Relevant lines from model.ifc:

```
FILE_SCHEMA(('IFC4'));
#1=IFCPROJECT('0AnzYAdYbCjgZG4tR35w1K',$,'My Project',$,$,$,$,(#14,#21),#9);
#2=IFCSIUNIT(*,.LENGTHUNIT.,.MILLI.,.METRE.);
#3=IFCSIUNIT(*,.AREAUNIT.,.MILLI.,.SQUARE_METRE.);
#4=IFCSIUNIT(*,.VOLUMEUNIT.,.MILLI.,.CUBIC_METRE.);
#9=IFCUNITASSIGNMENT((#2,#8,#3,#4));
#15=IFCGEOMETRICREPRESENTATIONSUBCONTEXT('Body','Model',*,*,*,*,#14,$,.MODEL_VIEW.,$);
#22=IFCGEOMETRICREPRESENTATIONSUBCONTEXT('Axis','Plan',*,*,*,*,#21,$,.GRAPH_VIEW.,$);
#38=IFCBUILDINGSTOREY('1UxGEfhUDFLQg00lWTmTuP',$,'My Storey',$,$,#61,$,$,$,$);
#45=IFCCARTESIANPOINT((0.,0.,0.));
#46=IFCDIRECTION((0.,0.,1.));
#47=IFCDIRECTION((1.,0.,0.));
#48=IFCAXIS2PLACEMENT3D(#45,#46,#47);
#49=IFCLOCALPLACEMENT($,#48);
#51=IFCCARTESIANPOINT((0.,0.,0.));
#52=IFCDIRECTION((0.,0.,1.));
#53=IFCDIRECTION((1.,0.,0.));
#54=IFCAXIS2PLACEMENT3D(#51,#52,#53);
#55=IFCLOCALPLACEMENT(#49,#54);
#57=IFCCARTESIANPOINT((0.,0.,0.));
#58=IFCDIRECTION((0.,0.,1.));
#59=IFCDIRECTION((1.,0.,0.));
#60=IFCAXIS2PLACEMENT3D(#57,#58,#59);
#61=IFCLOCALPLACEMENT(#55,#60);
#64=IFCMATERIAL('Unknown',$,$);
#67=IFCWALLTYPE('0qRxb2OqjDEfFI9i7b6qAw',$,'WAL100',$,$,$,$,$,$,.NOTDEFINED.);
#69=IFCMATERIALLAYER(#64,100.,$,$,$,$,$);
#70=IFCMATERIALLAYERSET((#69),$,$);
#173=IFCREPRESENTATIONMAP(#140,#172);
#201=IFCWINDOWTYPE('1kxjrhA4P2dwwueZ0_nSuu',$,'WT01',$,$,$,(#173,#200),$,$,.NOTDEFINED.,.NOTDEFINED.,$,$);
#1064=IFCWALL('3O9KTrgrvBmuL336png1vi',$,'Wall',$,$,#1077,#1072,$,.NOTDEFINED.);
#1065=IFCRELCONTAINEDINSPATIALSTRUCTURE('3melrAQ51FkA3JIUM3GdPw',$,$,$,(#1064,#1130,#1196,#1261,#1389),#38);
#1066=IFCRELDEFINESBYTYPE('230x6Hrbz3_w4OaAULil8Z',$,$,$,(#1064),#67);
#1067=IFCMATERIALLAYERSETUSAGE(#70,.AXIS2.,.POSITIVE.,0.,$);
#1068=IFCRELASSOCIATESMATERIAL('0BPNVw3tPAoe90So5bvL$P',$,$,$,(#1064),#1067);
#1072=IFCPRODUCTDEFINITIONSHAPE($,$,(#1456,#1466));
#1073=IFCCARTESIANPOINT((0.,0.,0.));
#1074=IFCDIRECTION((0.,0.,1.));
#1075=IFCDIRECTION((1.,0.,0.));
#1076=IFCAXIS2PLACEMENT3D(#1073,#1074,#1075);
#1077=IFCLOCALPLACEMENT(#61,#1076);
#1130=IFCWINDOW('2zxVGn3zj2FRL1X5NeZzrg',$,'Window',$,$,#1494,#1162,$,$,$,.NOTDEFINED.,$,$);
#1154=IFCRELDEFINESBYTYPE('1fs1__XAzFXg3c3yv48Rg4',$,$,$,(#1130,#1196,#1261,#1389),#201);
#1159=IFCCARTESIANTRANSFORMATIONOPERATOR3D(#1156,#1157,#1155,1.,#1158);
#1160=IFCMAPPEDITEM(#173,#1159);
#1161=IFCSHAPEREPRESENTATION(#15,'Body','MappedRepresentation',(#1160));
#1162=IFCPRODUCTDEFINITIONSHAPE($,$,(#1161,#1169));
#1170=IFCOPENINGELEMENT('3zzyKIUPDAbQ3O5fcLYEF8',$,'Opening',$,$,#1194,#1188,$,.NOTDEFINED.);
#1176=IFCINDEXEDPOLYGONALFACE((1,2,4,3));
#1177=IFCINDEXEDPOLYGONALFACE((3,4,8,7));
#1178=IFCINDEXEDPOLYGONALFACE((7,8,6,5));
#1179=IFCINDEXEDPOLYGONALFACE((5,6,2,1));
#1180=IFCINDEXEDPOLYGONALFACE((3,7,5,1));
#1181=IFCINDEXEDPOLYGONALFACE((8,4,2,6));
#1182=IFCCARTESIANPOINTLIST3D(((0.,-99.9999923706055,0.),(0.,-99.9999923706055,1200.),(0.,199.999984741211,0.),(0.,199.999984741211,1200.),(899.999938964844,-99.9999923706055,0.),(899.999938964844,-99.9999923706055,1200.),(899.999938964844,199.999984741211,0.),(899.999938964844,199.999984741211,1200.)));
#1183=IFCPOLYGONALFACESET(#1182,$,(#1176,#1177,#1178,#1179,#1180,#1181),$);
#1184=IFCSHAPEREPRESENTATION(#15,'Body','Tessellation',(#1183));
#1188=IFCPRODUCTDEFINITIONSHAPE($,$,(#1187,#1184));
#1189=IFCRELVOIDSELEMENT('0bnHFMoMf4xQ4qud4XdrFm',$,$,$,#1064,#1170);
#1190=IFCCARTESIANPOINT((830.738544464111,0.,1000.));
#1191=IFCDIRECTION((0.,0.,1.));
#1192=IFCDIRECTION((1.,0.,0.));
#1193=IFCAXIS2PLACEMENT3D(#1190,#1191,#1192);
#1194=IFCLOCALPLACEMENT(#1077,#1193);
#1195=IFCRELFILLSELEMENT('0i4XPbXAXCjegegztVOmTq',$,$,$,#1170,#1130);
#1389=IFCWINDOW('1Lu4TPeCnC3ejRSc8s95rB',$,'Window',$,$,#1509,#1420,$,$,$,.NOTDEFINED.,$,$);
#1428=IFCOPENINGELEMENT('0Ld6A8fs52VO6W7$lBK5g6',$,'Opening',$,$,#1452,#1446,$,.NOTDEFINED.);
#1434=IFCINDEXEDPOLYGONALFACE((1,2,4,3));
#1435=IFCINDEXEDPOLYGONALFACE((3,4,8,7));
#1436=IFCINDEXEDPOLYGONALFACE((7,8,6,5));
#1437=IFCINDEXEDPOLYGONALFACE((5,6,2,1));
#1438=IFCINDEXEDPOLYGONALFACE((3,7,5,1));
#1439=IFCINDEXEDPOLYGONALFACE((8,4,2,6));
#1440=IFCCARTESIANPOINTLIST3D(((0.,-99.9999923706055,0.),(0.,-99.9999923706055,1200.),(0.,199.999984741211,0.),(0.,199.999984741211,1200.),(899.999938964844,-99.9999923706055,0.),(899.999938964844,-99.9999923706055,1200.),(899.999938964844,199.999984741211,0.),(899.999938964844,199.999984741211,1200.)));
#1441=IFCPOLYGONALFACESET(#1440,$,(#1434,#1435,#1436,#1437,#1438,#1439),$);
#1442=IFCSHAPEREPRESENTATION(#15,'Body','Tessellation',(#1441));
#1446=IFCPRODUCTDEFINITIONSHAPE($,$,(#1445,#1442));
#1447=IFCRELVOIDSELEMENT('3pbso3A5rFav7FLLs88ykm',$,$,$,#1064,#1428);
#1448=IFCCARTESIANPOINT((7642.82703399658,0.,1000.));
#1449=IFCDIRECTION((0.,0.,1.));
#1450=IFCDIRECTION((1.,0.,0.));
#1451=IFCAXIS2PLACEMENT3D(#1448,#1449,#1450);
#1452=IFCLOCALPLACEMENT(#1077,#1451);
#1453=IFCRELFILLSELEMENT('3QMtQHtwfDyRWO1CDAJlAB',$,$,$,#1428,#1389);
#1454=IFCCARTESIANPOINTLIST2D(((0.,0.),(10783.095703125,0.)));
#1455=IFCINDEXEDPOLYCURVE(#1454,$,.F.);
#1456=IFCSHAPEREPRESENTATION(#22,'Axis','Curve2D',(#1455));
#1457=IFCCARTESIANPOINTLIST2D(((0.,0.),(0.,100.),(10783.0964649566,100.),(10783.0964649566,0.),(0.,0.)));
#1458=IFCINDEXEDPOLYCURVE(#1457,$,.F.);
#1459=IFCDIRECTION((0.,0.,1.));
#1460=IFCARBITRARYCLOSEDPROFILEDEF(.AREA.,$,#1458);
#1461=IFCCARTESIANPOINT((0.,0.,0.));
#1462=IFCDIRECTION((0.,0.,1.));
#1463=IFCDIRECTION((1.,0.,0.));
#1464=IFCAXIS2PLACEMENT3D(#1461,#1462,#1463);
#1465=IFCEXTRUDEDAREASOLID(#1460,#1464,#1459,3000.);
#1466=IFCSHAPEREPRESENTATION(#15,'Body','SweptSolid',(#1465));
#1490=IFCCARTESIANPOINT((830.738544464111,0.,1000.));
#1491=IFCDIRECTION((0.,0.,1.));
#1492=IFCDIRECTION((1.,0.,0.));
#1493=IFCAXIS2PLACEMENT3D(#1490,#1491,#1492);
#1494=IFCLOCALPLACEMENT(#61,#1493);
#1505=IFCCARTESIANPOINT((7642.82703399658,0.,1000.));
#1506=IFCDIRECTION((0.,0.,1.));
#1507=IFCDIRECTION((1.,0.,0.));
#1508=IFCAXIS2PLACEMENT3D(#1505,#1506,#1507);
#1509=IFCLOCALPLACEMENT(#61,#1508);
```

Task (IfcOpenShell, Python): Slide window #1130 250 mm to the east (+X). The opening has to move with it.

```python
import ifcopenshell
import ifcopenshell.api.geometry
import ifcopenshell.util.placement

model = ifcopenshell.open("model.ifc")

window = model.by_guid("2zxVGn3zj2FRL1X5NeZzrg")
opening = window.FillsVoids[0].RelatingOpeningElement
wall = opening.VoidsElements[0].RelatingBuildingElement

wall_matrix = ifcopenshell.util.placement.get_local_placement(wall.ObjectPlacement)
shift = wall_matrix[:3, 0] * 250.0
before = ifcopenshell.util.placement.get_local_placement(window.ObjectPlacement)[:3, 3].copy()

# The window is not placed relative to its opening, so move both.
for product in (opening, window):
    matrix = ifcopenshell.util.placement.get_local_placement(product.ObjectPlacement)
    matrix[:3, 3] += shift
    ifcopenshell.api.geometry.edit_object_placement(model, product=product, matrix=matrix, is_si=False)

after = ifcopenshell.util.placement.get_local_placement(window.ObjectPlacement)[:3, 3]
print("window moved by", (after - before).round(3) + 0.0)

model.write("model_rev.ifc")
```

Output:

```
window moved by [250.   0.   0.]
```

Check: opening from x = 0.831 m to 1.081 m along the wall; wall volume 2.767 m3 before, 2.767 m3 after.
